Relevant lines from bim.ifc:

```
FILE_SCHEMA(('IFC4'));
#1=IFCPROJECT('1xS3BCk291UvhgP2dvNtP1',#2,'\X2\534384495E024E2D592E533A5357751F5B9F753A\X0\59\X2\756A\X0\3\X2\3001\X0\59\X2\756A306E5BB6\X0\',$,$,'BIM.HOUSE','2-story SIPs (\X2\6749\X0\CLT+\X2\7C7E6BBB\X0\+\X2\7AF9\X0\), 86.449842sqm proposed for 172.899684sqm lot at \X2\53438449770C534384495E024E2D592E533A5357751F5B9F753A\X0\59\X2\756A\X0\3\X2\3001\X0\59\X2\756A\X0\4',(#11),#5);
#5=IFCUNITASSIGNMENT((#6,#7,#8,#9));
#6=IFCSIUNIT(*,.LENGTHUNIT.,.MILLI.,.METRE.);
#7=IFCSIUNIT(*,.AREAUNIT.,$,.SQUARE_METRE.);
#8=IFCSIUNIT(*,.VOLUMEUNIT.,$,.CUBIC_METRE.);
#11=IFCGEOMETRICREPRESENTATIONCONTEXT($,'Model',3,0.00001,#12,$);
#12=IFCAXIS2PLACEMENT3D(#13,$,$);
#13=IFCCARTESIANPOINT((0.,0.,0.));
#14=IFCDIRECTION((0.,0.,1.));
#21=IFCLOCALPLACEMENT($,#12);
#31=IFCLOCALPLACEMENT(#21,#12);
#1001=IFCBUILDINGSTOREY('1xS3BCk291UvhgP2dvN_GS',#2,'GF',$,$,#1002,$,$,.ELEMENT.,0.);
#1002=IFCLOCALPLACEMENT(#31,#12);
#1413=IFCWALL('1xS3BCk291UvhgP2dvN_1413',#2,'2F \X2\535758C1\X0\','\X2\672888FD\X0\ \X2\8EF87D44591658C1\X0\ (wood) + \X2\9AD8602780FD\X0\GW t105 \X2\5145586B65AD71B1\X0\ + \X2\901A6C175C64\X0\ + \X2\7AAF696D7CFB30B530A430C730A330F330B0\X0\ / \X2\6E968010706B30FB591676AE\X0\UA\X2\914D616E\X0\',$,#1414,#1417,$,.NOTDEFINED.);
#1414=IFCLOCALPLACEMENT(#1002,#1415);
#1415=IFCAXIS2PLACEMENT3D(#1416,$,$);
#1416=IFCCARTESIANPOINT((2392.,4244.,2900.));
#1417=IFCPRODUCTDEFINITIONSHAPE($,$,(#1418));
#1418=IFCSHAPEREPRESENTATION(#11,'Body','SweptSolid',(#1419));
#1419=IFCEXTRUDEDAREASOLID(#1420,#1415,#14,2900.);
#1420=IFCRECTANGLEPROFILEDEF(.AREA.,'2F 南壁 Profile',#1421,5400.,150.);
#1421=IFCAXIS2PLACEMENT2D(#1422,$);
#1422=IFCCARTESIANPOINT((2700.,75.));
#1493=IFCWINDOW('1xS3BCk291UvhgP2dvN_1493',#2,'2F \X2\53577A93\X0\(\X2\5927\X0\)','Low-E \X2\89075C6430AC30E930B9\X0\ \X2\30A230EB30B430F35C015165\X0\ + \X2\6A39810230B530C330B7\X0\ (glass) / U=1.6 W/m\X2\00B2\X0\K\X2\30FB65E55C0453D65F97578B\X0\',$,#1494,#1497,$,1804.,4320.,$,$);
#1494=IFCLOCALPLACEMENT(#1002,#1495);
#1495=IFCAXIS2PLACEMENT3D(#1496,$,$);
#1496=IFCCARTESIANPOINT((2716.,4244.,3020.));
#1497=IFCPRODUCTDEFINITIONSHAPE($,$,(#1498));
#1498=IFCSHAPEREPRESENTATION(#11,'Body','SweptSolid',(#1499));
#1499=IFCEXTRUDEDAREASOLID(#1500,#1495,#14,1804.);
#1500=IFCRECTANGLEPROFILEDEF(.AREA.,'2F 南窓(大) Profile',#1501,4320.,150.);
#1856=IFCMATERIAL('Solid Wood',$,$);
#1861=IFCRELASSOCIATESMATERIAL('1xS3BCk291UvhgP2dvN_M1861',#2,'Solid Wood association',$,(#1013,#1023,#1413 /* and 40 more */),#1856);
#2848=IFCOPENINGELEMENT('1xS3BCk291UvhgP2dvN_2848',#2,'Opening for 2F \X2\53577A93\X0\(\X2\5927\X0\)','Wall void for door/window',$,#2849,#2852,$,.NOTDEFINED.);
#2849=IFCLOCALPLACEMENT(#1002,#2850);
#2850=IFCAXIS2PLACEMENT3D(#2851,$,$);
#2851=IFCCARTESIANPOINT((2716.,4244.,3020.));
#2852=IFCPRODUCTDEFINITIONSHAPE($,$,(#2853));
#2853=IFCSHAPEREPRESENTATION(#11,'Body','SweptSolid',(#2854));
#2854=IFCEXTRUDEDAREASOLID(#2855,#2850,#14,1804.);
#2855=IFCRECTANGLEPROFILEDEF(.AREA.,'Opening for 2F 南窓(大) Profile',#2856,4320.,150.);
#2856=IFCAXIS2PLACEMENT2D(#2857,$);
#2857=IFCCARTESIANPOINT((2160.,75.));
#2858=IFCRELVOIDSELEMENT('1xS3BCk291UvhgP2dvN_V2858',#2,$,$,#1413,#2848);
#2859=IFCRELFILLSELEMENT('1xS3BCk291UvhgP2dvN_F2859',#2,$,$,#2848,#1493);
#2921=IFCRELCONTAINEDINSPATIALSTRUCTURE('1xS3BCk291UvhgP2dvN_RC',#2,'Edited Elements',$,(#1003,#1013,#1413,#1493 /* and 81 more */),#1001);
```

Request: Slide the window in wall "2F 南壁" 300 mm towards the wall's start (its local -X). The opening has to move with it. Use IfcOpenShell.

```python
import ifcopenshell
import ifcopenshell.api.geometry
import ifcopenshell.util.placement
import ifcopenshell.util.unit

model = ifcopenshell.open("bim.ifc")
unit_scale = ifcopenshell.util.unit.calculate_unit_scale(model)

window = model.by_guid("1xS3BCk291UvhgP2dvN_1493")
opening = window.FillsVoids[0].RelatingOpeningElement
wall = opening.VoidsElements[0].RelatingBuildingElement

wall_matrix = ifcopenshell.util.placement.get_local_placement(wall.ObjectPlacement)
shift = wall_matrix[:3, 0] * -0.3 / unit_scale
before = ifcopenshell.util.placement.get_local_placement(window.ObjectPlacement)[:3, 3].copy()

# The window is not placed relative to its opening, so move both.
for product in (opening, window):
    matrix = ifcopenshell.util.placement.get_local_placement(product.ObjectPlacement)
    matrix[:3, 3] += shift
    ifcopenshell.api.geometry.edit_object_placement(model, product=product, matrix=matrix, is_si=False)

after = ifcopenshell.util.placement.get_local_placement(window.ObjectPlacement)[:3, 3]
print("window moved by", (after - before).round(3) + 0.0)

model.write("bim_rev.ifc")
```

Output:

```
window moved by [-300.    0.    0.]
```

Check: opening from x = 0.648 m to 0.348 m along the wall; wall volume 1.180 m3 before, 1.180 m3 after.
